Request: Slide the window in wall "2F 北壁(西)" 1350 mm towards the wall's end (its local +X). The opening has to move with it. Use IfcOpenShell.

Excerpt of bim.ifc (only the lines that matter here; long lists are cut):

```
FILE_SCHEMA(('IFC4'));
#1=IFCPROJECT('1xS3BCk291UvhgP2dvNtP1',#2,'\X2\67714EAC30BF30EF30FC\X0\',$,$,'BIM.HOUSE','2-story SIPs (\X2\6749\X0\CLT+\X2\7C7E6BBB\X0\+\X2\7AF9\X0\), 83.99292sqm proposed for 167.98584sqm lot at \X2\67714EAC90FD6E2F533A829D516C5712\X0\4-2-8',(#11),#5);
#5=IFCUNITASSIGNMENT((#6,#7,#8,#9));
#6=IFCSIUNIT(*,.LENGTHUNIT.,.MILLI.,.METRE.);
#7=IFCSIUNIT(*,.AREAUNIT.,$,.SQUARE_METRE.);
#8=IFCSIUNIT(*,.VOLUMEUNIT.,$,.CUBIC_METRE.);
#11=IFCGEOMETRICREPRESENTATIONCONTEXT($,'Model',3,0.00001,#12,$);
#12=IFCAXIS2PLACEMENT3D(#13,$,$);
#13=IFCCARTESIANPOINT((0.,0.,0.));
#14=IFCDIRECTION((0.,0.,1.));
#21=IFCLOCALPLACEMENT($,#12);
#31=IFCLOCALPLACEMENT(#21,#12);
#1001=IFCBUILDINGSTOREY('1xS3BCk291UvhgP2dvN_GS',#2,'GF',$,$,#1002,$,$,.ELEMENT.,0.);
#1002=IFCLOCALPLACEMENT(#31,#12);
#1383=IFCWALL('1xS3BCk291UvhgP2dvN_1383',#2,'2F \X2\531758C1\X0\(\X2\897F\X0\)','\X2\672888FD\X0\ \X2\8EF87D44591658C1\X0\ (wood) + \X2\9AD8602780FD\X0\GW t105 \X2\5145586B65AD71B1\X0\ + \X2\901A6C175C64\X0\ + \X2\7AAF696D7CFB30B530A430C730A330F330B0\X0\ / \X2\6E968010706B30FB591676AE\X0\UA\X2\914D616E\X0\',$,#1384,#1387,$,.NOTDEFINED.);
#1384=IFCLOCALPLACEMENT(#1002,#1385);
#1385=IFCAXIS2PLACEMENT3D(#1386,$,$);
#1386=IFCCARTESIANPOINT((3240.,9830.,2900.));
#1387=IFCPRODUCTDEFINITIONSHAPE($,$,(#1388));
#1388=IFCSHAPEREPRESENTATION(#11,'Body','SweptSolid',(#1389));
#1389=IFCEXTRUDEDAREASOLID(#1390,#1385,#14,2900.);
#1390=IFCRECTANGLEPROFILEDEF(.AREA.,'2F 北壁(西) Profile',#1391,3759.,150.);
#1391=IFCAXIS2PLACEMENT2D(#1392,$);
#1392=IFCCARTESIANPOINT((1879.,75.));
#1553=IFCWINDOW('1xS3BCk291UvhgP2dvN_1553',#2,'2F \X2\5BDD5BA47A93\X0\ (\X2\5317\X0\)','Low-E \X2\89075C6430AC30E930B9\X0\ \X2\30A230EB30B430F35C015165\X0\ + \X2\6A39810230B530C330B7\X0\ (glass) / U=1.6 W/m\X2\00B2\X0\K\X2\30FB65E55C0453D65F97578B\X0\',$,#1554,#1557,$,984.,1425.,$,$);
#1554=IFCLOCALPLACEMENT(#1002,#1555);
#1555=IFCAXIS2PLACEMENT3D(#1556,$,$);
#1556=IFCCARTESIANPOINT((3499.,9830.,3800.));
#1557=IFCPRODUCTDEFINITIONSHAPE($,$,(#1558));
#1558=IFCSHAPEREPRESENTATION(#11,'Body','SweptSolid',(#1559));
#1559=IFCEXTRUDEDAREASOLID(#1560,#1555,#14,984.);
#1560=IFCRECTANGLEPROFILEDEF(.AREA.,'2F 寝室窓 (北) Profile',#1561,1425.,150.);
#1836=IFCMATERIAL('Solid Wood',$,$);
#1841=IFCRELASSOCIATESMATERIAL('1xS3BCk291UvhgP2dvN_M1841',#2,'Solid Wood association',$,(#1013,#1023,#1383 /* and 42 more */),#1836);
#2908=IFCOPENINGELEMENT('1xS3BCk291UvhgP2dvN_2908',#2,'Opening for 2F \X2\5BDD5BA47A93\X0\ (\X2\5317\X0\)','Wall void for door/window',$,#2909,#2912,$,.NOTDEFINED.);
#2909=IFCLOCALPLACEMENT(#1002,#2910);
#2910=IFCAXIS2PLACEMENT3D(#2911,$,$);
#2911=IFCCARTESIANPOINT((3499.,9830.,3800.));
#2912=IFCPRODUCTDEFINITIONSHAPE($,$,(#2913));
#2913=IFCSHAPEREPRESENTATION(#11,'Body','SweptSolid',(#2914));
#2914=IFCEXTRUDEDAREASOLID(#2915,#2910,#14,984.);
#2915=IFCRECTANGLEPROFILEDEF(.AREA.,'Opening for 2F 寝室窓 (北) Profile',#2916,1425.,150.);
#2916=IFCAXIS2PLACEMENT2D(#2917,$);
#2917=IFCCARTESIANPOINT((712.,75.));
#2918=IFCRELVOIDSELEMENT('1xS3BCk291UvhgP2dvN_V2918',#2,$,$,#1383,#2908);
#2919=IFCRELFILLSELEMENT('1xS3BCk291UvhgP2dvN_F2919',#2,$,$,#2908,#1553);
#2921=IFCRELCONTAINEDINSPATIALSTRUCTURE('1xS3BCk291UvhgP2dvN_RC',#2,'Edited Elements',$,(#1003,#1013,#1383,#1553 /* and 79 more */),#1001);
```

```python
import ifcopenshell
import ifcopenshell.api.geometry
import ifcopenshell.util.placement
import ifcopenshell.util.unit

model = ifcopenshell.open("bim.ifc")
unit_scale = ifcopenshell.util.unit.calculate_unit_scale(model)

window = model.by_guid("1xS3BCk291UvhgP2dvN_1553")
opening = window.FillsVoids[0].RelatingOpeningElement
wall = opening.VoidsElements[0].RelatingBuildingElement

wall_matrix = ifcopenshell.util.placement.get_local_placement(wall.ObjectPlacement)
shift = wall_matrix[:3, 0] * 1.35 / unit_scale
before = ifcopenshell.util.placement.get_local_placement(window.ObjectPlacement)[:3, 3].copy()

# The window is not placed relative to its opening, so move both.
for product in (opening, window):
    matrix = ifcopenshell.util.placement.get_local_placement(product.ObjectPlacement)
    matrix[:3, 3] += shift
    ifcopenshell.api.geometry.edit_object_placement(model, product=product, matrix=matrix, is_si=False)

after = ifcopenshell.util.placement.get_local_placement(window.ObjectPlacement)[:3, 3]
print("window moved by", (after - before).round(3) + 0.0)

model.write("bim_rev.ifc")
```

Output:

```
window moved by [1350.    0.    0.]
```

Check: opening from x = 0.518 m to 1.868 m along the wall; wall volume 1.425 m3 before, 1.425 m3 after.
